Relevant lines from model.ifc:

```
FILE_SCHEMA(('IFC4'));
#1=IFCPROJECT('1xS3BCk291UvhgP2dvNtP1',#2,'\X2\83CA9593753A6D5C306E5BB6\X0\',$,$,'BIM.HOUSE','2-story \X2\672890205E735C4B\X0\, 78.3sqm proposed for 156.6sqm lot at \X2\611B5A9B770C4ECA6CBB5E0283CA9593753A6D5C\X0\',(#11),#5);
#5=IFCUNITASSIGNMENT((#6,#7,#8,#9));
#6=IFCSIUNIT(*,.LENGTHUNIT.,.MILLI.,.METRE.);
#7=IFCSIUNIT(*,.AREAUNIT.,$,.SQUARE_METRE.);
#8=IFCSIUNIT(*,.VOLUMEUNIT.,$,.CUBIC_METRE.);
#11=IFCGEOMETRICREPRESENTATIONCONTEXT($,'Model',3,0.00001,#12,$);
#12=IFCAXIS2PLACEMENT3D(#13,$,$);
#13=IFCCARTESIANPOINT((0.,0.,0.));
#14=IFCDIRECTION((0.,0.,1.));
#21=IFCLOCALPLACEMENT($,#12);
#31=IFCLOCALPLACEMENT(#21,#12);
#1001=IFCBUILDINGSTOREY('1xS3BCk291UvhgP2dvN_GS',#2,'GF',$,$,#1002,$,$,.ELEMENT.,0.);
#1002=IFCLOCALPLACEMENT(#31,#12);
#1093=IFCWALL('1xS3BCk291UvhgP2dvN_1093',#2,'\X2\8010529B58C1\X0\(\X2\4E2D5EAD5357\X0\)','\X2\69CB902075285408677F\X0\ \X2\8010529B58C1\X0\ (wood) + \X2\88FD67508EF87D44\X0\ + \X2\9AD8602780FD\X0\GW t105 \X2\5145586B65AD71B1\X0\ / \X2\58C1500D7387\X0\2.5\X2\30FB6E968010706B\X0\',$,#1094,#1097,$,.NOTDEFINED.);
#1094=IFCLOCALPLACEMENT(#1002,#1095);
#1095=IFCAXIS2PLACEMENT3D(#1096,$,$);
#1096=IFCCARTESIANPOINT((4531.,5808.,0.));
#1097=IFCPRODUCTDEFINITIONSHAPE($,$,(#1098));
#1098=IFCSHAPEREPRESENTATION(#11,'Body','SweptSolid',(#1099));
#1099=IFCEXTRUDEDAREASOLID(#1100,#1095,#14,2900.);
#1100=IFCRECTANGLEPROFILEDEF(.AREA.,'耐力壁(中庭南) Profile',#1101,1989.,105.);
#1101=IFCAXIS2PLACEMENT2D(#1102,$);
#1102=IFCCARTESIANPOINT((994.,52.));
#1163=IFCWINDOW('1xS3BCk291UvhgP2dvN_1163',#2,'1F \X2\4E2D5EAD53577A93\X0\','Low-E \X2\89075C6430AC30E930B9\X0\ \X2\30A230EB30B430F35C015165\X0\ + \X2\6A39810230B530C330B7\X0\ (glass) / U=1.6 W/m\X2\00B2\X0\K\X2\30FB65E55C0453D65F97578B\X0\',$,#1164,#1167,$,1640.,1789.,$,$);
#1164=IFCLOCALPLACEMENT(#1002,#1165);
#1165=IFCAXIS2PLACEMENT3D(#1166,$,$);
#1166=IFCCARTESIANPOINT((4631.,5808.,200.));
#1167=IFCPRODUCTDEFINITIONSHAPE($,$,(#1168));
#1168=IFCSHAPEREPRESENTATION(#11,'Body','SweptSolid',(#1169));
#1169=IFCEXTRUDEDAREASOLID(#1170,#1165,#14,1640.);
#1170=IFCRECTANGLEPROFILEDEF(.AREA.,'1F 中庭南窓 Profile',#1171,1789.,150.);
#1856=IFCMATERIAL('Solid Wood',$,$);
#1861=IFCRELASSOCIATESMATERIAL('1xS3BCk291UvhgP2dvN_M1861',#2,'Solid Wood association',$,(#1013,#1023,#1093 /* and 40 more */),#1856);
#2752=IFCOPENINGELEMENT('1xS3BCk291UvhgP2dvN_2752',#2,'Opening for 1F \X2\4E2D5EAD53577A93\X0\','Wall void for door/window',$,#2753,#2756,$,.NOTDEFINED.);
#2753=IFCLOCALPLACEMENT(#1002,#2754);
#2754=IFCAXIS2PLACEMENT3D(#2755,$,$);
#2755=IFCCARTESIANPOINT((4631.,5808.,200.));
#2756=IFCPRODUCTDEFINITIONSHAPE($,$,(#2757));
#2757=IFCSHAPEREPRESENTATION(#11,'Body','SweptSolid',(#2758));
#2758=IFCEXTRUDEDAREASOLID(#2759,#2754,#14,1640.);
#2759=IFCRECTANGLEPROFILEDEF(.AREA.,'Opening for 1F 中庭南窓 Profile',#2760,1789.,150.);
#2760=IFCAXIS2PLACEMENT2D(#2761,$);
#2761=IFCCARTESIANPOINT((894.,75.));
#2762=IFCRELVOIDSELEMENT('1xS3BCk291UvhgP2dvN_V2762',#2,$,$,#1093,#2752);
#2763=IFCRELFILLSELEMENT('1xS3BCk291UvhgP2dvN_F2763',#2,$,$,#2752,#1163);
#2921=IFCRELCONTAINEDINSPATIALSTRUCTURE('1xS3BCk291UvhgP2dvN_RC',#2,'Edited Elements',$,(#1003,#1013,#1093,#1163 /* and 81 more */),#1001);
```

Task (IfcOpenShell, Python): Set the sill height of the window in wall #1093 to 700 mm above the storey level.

```python
import numpy as np
import ifcopenshell
import ifcopenshell.api.geometry
import ifcopenshell.geom
import ifcopenshell.util.element
import ifcopenshell.util.placement
import ifcopenshell.util.shape
import ifcopenshell.util.unit

model = ifcopenshell.open("model.ifc")
unit_scale = ifcopenshell.util.unit.calculate_unit_scale(model)

window = model.by_guid("1xS3BCk291UvhgP2dvN_1163")
opening = window.FillsVoids[0].RelatingOpeningElement
storey = ifcopenshell.util.element.get_container(window, ifc_class="IfcBuildingStorey")
level = ifcopenshell.util.placement.get_local_placement(storey.ObjectPlacement)[2, 3]

# The opening's origin need not be at the sill, so measure its lowest point.
shape = ifcopenshell.geom.create_shape(ifcopenshell.geom.settings(), opening)
bottom = ifcopenshell.util.shape.get_shape_bottom_elevation(shape, shape.geometry) / unit_scale
dz = level + 700.0 - bottom

shift = np.array([0.0, 0.0, dz])
# The window is not placed relative to its opening, so move both.
for product in (opening, window):
    matrix = ifcopenshell.util.placement.get_local_placement(product.ObjectPlacement)
    matrix[:3, 3] += shift
    ifcopenshell.api.geometry.edit_object_placement(model, product=product, matrix=matrix, is_si=False)

print(f"moved by {dz * unit_scale:+.3f} m")

model.write("model_rev.ifc")
```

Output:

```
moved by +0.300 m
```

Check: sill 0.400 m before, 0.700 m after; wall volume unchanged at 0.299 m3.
